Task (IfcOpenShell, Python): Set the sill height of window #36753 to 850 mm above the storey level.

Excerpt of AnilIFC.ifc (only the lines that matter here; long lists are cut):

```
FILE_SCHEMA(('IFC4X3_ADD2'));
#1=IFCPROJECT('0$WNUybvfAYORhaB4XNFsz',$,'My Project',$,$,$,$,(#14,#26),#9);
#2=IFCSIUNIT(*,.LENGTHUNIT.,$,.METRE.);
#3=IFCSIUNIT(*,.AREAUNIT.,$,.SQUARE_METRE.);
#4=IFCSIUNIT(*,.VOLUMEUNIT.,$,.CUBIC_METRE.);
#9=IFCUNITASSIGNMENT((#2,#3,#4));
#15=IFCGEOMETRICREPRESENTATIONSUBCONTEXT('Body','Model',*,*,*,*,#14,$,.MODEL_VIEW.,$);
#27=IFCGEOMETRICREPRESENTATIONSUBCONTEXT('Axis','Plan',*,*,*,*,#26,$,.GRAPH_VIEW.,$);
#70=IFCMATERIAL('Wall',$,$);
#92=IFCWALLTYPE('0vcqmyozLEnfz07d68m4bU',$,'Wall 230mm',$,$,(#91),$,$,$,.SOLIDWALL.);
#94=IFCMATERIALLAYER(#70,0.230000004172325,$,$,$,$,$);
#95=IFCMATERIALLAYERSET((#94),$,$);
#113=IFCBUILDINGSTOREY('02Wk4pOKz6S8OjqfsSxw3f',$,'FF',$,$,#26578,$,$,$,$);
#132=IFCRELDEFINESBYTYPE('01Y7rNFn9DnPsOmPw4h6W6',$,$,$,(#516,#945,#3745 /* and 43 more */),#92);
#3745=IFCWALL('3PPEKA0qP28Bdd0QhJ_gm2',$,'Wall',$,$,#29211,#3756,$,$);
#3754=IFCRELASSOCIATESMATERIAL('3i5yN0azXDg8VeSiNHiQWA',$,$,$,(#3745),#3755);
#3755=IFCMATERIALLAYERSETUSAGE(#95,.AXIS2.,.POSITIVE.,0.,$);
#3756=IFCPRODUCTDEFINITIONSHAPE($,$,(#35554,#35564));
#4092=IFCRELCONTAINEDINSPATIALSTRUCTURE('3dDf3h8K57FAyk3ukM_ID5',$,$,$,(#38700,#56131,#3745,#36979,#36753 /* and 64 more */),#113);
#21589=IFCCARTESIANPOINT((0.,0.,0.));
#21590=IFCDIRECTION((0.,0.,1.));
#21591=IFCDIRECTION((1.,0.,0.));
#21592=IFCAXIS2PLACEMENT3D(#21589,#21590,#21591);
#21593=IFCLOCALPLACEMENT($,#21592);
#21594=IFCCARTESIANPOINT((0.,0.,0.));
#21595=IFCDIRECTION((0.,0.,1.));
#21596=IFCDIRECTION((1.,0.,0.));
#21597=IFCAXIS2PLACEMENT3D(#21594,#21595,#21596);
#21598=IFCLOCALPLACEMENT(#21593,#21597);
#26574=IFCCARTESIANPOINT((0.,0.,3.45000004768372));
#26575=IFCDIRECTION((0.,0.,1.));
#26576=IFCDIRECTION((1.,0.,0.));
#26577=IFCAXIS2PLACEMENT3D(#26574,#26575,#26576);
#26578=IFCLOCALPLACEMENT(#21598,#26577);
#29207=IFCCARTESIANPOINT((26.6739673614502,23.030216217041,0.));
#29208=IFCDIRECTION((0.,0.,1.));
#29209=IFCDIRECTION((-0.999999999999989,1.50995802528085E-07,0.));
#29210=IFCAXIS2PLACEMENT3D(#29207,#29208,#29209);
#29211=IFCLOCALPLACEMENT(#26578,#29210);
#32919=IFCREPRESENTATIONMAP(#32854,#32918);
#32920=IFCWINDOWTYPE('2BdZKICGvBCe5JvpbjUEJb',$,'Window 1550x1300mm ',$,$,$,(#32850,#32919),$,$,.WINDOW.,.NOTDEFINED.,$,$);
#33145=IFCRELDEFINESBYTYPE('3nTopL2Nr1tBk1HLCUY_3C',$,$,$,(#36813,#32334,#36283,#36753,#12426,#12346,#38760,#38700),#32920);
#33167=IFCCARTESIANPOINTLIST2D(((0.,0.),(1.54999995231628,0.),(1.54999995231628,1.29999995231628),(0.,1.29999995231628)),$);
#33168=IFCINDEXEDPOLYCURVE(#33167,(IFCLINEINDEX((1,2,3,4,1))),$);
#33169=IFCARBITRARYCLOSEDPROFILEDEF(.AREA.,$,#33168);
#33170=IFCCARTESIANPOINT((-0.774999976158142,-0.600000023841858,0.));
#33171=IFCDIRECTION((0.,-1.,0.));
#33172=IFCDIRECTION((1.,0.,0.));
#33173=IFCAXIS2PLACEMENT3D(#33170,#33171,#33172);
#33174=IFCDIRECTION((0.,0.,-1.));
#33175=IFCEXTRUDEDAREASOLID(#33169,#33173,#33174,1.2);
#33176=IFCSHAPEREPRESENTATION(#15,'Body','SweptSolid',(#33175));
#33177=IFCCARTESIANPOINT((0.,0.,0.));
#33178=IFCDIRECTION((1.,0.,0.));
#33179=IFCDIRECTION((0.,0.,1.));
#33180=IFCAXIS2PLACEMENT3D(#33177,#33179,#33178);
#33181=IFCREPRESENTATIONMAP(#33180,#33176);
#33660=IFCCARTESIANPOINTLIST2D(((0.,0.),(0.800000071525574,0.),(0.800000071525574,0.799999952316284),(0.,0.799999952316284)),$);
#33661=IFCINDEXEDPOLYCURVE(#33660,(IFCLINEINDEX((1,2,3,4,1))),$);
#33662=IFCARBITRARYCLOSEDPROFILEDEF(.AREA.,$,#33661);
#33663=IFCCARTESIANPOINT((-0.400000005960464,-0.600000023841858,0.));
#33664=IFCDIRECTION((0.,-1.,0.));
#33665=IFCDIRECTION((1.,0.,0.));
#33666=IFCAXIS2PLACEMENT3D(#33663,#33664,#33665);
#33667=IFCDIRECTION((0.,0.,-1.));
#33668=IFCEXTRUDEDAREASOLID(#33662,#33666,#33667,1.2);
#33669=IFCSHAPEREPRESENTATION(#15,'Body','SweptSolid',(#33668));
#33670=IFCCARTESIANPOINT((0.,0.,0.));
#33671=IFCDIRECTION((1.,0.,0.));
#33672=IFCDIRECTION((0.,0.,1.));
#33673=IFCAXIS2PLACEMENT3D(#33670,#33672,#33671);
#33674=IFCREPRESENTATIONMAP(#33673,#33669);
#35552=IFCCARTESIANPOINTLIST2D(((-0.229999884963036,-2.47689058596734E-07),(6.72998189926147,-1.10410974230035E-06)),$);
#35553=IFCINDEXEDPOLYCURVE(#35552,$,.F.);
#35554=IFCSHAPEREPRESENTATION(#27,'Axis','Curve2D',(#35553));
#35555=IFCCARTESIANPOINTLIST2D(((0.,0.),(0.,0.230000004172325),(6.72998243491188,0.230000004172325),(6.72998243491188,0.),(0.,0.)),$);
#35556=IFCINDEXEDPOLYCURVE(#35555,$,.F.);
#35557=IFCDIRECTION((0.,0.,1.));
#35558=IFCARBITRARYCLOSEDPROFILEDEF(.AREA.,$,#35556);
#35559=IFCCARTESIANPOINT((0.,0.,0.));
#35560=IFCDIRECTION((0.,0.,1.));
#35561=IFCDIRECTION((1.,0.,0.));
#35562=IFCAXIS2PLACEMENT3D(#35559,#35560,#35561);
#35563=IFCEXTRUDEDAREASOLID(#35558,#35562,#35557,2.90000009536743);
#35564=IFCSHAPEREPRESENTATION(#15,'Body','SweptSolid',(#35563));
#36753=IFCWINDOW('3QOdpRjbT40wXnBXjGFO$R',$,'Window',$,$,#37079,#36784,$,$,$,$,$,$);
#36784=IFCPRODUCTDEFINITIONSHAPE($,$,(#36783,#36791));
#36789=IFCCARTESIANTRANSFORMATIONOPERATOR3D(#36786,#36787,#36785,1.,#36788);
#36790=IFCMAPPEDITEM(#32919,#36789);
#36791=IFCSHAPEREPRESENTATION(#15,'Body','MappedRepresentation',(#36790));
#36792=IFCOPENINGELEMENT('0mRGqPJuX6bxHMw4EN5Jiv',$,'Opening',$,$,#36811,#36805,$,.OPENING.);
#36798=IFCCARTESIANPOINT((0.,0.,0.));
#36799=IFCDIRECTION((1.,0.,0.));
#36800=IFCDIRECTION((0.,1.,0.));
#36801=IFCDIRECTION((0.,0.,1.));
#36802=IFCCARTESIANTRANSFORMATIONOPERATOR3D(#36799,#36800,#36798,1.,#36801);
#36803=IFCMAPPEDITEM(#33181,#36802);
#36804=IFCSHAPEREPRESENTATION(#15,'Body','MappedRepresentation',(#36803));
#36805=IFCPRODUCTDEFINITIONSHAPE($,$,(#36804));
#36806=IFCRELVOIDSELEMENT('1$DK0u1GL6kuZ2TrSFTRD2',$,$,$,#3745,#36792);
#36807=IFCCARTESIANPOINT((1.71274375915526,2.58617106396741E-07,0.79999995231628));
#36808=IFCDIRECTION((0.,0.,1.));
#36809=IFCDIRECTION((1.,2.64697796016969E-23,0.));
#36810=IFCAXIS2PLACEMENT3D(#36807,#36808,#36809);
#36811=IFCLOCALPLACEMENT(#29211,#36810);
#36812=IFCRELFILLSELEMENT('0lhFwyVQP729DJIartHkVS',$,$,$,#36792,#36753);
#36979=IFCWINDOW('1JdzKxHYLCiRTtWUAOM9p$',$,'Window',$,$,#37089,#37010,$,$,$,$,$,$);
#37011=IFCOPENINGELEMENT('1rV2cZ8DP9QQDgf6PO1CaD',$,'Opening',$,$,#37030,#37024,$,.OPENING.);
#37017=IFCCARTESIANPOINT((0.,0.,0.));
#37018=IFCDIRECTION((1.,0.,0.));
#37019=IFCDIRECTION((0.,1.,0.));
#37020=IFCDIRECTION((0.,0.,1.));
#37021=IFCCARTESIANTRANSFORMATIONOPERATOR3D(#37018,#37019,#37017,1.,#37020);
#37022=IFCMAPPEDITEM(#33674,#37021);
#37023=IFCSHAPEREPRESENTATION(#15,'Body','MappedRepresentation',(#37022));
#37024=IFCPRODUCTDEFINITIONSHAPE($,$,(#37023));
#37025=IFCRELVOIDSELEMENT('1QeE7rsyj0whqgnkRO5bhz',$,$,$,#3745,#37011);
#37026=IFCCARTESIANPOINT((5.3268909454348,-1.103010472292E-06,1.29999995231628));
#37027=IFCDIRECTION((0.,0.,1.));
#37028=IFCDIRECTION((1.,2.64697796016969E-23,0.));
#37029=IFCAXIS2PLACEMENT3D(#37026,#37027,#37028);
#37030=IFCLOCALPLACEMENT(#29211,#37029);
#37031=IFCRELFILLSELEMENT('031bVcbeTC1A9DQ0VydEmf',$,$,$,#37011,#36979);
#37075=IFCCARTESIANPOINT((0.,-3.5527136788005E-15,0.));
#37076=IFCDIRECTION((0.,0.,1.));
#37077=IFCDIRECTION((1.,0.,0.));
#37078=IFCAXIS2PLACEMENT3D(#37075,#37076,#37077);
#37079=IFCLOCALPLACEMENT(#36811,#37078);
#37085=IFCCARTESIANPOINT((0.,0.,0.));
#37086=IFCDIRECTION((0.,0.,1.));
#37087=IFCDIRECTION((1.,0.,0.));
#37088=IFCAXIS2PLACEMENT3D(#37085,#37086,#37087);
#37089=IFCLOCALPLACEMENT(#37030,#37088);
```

```python
import numpy as np
import ifcopenshell
import ifcopenshell.api.geometry
import ifcopenshell.geom
import ifcopenshell.util.element
import ifcopenshell.util.placement
import ifcopenshell.util.shape
import ifcopenshell.util.unit

model = ifcopenshell.open("AnilIFC.ifc")
unit_scale = ifcopenshell.util.unit.calculate_unit_scale(model)

window = model.by_guid("3QOdpRjbT40wXnBXjGFO$R")
opening = window.FillsVoids[0].RelatingOpeningElement
storey = ifcopenshell.util.element.get_container(window, ifc_class="IfcBuildingStorey")
level = ifcopenshell.util.placement.get_local_placement(storey.ObjectPlacement)[2, 3]

# The opening's origin need not be at the sill, so measure its lowest point.
shape = ifcopenshell.geom.create_shape(ifcopenshell.geom.settings(), opening)
bottom = ifcopenshell.util.shape.get_shape_bottom_elevation(shape, shape.geometry) / unit_scale
dz = level + 0.85 - bottom

shift = np.array([0.0, 0.0, dz])
# The window is placed relative to its opening, so it follows when the opening moves.
matrix = ifcopenshell.util.placement.get_local_placement(opening.ObjectPlacement)
matrix[:3, 3] += shift
ifcopenshell.api.geometry.edit_object_placement(
    model, product=opening, matrix=matrix, is_si=False, should_transform_children=True
)

print(f"moved by {dz * unit_scale:+.3f} m")

model.write("AnilIFC_updated.ifc")
```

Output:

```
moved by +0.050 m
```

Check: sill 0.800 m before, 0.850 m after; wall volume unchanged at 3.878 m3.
